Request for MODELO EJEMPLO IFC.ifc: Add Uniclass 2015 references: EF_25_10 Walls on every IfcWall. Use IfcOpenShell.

First a look at what the model holds.

```python
import ifcopenshell

model = ifcopenshell.open("MODELO EJEMPLO IFC.ifc")
print(model.schema)
print("classifications:", [c.Name for c in model.by_type("IfcClassification")])
for ifc_class in ("IfcDoor", "IfcRoof", "IfcStair", "IfcWall", "IfcWindow"):
    print(ifc_class, len(model.by_type(ifc_class)))
```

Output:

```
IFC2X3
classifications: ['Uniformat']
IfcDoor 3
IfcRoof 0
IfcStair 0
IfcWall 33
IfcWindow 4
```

```python
import ifcopenshell
import ifcopenshell.api.classification

model = ifcopenshell.open("MODELO EJEMPLO IFC.ifc")

# IFC2X3 requires Source and Edition and has no link from the project to the system.
system = model.create_entity("IfcClassification", Source="NBS", Edition="2015", Name="Uniclass 2015")

codes = {
    "IfcWall": ("EF_25_10", "Walls"),
}
for ifc_class, (code, name) in codes.items():
    products = model.by_type(ifc_class)
    ifcopenshell.api.classification.add_reference(
        model, products=products, classification=system, identification=code, name=name
    )
    print(code, len(products))

model.write("MODELO EJEMPLO IFC_edited.ifc")
```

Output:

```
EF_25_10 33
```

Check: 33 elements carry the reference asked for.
